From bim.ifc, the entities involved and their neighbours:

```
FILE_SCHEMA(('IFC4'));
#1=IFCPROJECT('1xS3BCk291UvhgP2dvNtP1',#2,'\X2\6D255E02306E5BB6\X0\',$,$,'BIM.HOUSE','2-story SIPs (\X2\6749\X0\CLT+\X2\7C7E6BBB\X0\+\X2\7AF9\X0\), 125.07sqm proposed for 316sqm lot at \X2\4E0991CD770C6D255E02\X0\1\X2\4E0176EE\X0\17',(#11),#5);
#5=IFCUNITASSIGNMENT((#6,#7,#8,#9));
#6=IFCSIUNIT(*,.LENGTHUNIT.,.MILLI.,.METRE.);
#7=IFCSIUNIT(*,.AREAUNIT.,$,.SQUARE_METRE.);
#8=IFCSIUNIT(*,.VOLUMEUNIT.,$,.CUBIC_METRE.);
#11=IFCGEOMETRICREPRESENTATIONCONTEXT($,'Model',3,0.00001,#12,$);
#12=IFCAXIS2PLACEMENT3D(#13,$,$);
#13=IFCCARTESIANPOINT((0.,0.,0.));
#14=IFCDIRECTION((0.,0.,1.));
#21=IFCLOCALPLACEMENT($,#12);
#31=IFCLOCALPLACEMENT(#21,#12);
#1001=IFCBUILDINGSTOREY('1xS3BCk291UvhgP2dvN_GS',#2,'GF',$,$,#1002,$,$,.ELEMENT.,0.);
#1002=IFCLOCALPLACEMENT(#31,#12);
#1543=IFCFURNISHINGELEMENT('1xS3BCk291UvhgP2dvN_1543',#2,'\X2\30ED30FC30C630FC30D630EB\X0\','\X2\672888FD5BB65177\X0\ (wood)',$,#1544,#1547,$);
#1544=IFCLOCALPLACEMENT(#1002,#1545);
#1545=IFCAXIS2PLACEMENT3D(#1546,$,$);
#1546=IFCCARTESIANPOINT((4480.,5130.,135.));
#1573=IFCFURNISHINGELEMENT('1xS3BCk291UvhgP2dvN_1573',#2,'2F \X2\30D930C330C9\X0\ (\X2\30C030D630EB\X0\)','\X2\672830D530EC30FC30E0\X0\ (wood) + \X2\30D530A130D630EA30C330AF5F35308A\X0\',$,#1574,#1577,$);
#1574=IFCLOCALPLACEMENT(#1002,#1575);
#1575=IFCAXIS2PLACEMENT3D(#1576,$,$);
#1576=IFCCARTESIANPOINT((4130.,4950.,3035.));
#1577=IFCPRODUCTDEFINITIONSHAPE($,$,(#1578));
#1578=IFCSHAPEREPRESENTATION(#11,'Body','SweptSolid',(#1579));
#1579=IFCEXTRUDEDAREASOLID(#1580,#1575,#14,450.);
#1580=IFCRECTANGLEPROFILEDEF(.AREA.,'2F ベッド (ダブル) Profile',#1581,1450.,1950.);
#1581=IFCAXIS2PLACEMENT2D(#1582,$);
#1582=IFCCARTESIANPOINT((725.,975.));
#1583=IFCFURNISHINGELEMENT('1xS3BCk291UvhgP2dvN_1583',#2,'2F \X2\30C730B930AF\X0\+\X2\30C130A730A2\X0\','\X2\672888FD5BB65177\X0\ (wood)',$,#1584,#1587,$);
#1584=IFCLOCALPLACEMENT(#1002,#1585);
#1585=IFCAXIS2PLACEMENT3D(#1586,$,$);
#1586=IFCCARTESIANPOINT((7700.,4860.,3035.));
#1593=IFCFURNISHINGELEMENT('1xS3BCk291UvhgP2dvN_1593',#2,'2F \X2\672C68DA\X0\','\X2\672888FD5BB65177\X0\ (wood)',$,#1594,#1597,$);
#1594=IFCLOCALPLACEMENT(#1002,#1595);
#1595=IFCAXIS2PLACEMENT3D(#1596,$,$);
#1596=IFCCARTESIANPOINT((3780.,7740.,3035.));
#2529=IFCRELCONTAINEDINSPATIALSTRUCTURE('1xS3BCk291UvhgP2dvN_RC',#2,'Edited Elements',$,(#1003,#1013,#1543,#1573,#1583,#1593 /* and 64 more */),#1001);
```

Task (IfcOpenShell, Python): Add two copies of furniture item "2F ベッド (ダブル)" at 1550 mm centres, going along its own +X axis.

```python
import ifcopenshell
import ifcopenshell.api.geometry
import ifcopenshell.api.root
import ifcopenshell.util.element
import ifcopenshell.util.placement

model = ifcopenshell.open("bim.ifc")


def reuse_history(source, copy):
    """copy_class also copies each property set's owner history, people and application; keep the originals."""
    for rel in copy.IsDefinedBy:
        if rel.is_a("IfcRelDefinesByProperties") and (history := rel.RelatingPropertyDefinition.OwnerHistory):
            rel.RelatingPropertyDefinition.OwnerHistory = source.OwnerHistory
            ifcopenshell.util.element.remove_deep2(model, history)


source = model.by_guid("1xS3BCk291UvhgP2dvN_1573")
base = ifcopenshell.util.placement.get_local_placement(source.ObjectPlacement)
step = base[:3, 0] * 1550.0

for i in range(1, 3):
    copy = ifcopenshell.api.root.copy_class(model, product=source)
    copy.Representation = ifcopenshell.util.element.copy_deep(
        model, source.Representation, exclude=["IfcGeometricRepresentationContext", "IfcRepresentationMap"]
    )
    reuse_history(source, copy)
    matrix = base.copy()
    matrix[:3, 3] += i * step
    print("added at", matrix[:3, 3].round(3) + 0.0)
    ifcopenshell.api.geometry.edit_object_placement(model, product=copy, matrix=matrix, is_si=False)

model.write("bim_edited.ifc")
```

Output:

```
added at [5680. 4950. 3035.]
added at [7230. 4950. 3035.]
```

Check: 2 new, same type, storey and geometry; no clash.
